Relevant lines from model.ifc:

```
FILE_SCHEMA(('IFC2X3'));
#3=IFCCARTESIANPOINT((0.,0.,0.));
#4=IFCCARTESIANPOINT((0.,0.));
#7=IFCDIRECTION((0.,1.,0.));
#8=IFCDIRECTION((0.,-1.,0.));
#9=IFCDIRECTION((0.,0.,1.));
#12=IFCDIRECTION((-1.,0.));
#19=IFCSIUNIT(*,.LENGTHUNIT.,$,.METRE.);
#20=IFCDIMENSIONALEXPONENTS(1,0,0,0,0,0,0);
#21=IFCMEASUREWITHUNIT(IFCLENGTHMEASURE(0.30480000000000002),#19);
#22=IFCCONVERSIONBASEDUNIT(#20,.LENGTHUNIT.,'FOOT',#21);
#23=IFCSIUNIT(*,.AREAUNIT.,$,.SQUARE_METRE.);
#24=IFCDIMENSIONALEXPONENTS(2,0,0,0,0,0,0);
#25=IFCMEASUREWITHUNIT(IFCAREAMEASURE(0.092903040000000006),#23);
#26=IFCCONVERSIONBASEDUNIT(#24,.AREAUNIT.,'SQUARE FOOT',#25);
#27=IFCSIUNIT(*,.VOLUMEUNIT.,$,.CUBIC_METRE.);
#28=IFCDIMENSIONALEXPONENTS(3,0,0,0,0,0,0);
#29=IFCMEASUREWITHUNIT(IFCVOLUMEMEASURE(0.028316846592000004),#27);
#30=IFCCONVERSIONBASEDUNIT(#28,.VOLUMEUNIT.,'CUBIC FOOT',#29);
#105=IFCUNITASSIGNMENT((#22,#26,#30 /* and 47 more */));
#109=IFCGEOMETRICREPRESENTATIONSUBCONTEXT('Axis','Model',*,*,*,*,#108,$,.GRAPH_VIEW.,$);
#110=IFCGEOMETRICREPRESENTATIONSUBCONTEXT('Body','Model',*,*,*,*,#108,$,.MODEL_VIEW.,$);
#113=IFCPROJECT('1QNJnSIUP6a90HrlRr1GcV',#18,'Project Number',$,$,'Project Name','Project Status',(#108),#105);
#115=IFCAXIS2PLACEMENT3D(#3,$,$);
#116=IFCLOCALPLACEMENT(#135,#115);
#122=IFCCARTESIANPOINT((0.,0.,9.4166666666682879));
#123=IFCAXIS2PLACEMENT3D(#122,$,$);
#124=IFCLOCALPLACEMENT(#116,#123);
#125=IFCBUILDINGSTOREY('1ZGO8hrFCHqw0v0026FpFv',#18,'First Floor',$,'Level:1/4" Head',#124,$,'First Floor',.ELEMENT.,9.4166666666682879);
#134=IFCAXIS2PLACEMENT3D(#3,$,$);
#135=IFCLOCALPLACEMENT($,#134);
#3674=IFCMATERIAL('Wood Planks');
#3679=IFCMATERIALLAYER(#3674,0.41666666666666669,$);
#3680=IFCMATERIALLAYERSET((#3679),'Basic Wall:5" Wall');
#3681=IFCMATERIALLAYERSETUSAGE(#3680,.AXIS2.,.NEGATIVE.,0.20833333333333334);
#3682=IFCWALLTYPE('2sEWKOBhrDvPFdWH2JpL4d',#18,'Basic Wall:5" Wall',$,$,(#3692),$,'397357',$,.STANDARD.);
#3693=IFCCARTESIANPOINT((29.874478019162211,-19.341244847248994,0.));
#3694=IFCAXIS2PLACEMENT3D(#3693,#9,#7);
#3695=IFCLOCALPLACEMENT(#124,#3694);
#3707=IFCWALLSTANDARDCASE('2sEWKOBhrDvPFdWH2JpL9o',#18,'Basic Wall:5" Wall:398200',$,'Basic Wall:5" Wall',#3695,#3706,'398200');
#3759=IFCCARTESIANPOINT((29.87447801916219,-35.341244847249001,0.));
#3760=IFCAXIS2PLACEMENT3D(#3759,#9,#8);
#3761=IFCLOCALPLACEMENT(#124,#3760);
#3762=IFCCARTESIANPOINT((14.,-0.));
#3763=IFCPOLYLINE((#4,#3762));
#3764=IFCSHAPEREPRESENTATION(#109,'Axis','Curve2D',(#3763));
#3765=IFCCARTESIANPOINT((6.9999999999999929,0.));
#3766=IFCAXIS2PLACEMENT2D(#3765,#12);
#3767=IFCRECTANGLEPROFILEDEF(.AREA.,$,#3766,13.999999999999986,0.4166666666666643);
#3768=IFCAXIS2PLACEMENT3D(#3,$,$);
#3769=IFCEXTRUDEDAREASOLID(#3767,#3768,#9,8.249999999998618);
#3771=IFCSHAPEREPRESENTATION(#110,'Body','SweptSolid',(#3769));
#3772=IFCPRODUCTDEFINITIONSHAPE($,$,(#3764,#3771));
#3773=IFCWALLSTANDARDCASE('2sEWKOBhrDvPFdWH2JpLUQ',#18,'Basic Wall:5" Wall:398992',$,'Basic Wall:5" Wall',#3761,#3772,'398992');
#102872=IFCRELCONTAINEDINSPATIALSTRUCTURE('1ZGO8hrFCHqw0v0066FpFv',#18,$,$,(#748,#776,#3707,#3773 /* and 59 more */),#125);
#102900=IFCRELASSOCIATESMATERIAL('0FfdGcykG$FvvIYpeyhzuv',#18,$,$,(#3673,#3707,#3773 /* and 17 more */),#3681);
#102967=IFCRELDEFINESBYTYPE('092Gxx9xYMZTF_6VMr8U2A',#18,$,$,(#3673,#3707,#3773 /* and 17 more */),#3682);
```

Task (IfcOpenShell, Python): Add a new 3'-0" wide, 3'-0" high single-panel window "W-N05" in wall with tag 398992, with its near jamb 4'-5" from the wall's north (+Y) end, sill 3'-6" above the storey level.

```python
import numpy as np
import ifcopenshell
import ifcopenshell.api.feature
import ifcopenshell.api.geometry
import ifcopenshell.api.root
import ifcopenshell.api.spatial
import ifcopenshell.api.type
import ifcopenshell.geom
import ifcopenshell.util.element
import ifcopenshell.util.placement
import ifcopenshell.util.representation
import ifcopenshell.util.shape
import ifcopenshell.util.unit

model = ifcopenshell.open("model.ifc")
unit_scale = ifcopenshell.util.unit.calculate_unit_scale(model)
settings = ifcopenshell.geom.settings()


def volume(element):
    """Net volume in cubic metres, openings subtracted."""
    shape = ifcopenshell.geom.create_shape(settings, element)
    return ifcopenshell.util.shape.get_volume(shape.geometry)


wall = model.by_id(3773)
storey = ifcopenshell.util.element.get_container(wall, ifc_class="IfcBuildingStorey")
context = ifcopenshell.util.representation.get_context(model, "Model", "Body", "MODEL_VIEW")
before = volume(wall)

width, height, from_end, sill = 0.9144, 0.9144, 1.3462, 1.0668  # metres

# The wall runs along its own X axis, and the end named is its -X end.
wall_shape = ifcopenshell.geom.create_shape(settings, wall)
x, y, z = ifcopenshell.util.shape.get_vertices(wall_shape.geometry).T
start = x.min() + from_end
face, thickness = float(y.min()), float(y.max() - y.min())
wall_matrix = ifcopenshell.util.placement.get_local_placement(wall.ObjectPlacement)
level = ifcopenshell.util.placement.get_local_placement(storey.ObjectPlacement)[2, 3]


def in_wall(x, y):
    """Placement at x, y metres in the wall's axes, at sill height."""
    matrix = wall_matrix.copy()
    matrix[:, 3] = wall_matrix @ np.array([x / unit_scale, y / unit_scale, 0.0, 1.0])
    matrix[2, 3] = level + sill / unit_scale
    return matrix


# Opening: a box that overshoots both wall faces by 50 mm.
opening = ifcopenshell.api.root.create_entity(model, ifc_class="IfcOpeningElement")
box = ifcopenshell.api.geometry.add_wall_representation(
    model, context=context, length=width, height=height, thickness=thickness + 0.1
)
ifcopenshell.api.geometry.assign_representation(model, product=opening, representation=box)
ifcopenshell.api.geometry.edit_object_placement(model, product=opening, matrix=in_wall(start, face - 0.05), is_si=False)
ifcopenshell.api.feature.add_feature(model, feature=opening, element=wall)

window = ifcopenshell.api.root.create_entity(model, ifc_class="IfcWindow", name="W-N05")
window.OverallWidth, window.OverallHeight = width / unit_scale, height / unit_scale
body = ifcopenshell.api.geometry.add_window_representation(
    model,
    context=context,
    overall_width=window.OverallWidth,
    overall_height=window.OverallHeight,
    partition_type="SINGLE_PANEL",
)
ifcopenshell.api.geometry.assign_representation(model, product=window, representation=body)
ifcopenshell.api.spatial.assign_container(model, products=[window], relating_structure=storey)
fills = ifcopenshell.api.feature.add_filling(model, opening=opening, element=window)
fills.OwnerHistory = window.OwnerHistory  # required in IFC2X3

# IFC2X3 keeps the operation on the window style.
style = ifcopenshell.api.root.create_entity(model, ifc_class="IfcWindowStyle", name="W-N05")
style.OperationType, style.ConstructionType = "SINGLE_PANEL", "NOTDEFINED"
style.ParameterTakesPrecedence = style.Sizeable = False
ifcopenshell.api.type.assign_type(model, related_objects=[window], relating_type=style)

# Centre the window in the wall's thickness.
ifcopenshell.api.geometry.edit_object_placement(model, product=window, matrix=in_wall(start, face), is_si=False)
window_shape = ifcopenshell.geom.create_shape(settings, window)
depth = ifcopenshell.util.shape.get_vertices(window_shape.geometry)[:, 1]
offset = face + thickness / 2 - (depth.min() + depth.max()) / 2
ifcopenshell.api.geometry.edit_object_placement(model, product=window, matrix=in_wall(start, offset), is_si=False)

after = volume(wall)

print(f"wall volume {before:.3f} -> {after:.3f} m3")

model.write("model_updated.ifc")
```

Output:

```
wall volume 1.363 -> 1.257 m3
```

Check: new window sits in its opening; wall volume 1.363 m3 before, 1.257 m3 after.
